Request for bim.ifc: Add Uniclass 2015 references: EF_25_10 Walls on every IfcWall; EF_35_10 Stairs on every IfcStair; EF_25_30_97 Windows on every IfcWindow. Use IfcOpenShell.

First a look at what the model holds.

```python
import ifcopenshell

model = ifcopenshell.open("bim.ifc")
print(model.schema)
print("classifications:", [c.Name for c in model.by_type("IfcClassification")])
for ifc_class in ("IfcDoor", "IfcRoof", "IfcStair", "IfcWall", "IfcWindow"):
    print(ifc_class, len(model.by_type(ifc_class)))
```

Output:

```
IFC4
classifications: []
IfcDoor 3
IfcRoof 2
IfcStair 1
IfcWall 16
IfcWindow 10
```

```python
import ifcopenshell
import ifcopenshell.api.classification

model = ifcopenshell.open("bim.ifc")

system = ifcopenshell.api.classification.add_classification(model, classification="Uniclass 2015")

codes = {
    "IfcWall": ("EF_25_10", "Walls"),
    "IfcStair": ("EF_35_10", "Stairs"),
    "IfcWindow": ("EF_25_30_97", "Windows"),
}
for ifc_class, (code, name) in codes.items():
    products = model.by_type(ifc_class)
    ifcopenshell.api.classification.add_reference(
        model, products=products, classification=system, identification=code, name=name
    )
    print(code, len(products))

model.write("bim-out.ifc")
```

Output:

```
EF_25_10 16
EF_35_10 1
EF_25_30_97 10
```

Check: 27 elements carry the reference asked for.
